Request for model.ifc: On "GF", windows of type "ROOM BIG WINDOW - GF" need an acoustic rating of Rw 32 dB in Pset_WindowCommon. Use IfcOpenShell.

First a look at what the model holds.

```python
import ifcopenshell
import ifcopenshell.util.element

model = ifcopenshell.open("model.ifc")
print(model.schema)
storey = next(s for s in model.by_type("IfcBuildingStorey") if s.Name == "GF")
windows = [e for e in ifcopenshell.util.element.get_decomposition(storey) if e.is_a("IfcWindow")]
seen = {}
for e in windows:
    element_type = ifcopenshell.util.element.get_type(e)
    key = (element_type.Name if element_type != e and element_type else None, ifcopenshell.util.element.get_pset(e, "Pset_WindowCommon", "AcousticRating"))
    seen[key] = seen.get(key, 0) + 1
for (name, value), count in sorted(seen.items(), key=str):
    print(count, "x", name, "|", value)
```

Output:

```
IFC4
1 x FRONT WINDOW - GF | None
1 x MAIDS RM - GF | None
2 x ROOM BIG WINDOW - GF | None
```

```python
import ifcopenshell
import ifcopenshell.api.pset
import ifcopenshell.util.element

model = ifcopenshell.open("model.ifc")

storey = next(s for s in model.by_type("IfcBuildingStorey") if s.Name == "GF")
windows = [e for e in ifcopenshell.util.element.get_decomposition(storey) if e.is_a("IfcWindow")]

count = 0
for e in windows:
    element_type = ifcopenshell.util.element.get_type(e)
    if element_type in (None, e) or element_type.Name != "ROOM BIG WINDOW - GF":
        continue
    # add_pset returns the element's existing set when there is one.
    pset = ifcopenshell.api.pset.add_pset(model, product=e, name="Pset_WindowCommon")
    ifcopenshell.api.pset.edit_pset(model, pset=pset, properties={"AcousticRating": "Rw 32 dB"})
    count += 1

print(count, "windows updated")

model.write("model_edited.ifc")
```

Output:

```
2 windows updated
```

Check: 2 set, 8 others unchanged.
